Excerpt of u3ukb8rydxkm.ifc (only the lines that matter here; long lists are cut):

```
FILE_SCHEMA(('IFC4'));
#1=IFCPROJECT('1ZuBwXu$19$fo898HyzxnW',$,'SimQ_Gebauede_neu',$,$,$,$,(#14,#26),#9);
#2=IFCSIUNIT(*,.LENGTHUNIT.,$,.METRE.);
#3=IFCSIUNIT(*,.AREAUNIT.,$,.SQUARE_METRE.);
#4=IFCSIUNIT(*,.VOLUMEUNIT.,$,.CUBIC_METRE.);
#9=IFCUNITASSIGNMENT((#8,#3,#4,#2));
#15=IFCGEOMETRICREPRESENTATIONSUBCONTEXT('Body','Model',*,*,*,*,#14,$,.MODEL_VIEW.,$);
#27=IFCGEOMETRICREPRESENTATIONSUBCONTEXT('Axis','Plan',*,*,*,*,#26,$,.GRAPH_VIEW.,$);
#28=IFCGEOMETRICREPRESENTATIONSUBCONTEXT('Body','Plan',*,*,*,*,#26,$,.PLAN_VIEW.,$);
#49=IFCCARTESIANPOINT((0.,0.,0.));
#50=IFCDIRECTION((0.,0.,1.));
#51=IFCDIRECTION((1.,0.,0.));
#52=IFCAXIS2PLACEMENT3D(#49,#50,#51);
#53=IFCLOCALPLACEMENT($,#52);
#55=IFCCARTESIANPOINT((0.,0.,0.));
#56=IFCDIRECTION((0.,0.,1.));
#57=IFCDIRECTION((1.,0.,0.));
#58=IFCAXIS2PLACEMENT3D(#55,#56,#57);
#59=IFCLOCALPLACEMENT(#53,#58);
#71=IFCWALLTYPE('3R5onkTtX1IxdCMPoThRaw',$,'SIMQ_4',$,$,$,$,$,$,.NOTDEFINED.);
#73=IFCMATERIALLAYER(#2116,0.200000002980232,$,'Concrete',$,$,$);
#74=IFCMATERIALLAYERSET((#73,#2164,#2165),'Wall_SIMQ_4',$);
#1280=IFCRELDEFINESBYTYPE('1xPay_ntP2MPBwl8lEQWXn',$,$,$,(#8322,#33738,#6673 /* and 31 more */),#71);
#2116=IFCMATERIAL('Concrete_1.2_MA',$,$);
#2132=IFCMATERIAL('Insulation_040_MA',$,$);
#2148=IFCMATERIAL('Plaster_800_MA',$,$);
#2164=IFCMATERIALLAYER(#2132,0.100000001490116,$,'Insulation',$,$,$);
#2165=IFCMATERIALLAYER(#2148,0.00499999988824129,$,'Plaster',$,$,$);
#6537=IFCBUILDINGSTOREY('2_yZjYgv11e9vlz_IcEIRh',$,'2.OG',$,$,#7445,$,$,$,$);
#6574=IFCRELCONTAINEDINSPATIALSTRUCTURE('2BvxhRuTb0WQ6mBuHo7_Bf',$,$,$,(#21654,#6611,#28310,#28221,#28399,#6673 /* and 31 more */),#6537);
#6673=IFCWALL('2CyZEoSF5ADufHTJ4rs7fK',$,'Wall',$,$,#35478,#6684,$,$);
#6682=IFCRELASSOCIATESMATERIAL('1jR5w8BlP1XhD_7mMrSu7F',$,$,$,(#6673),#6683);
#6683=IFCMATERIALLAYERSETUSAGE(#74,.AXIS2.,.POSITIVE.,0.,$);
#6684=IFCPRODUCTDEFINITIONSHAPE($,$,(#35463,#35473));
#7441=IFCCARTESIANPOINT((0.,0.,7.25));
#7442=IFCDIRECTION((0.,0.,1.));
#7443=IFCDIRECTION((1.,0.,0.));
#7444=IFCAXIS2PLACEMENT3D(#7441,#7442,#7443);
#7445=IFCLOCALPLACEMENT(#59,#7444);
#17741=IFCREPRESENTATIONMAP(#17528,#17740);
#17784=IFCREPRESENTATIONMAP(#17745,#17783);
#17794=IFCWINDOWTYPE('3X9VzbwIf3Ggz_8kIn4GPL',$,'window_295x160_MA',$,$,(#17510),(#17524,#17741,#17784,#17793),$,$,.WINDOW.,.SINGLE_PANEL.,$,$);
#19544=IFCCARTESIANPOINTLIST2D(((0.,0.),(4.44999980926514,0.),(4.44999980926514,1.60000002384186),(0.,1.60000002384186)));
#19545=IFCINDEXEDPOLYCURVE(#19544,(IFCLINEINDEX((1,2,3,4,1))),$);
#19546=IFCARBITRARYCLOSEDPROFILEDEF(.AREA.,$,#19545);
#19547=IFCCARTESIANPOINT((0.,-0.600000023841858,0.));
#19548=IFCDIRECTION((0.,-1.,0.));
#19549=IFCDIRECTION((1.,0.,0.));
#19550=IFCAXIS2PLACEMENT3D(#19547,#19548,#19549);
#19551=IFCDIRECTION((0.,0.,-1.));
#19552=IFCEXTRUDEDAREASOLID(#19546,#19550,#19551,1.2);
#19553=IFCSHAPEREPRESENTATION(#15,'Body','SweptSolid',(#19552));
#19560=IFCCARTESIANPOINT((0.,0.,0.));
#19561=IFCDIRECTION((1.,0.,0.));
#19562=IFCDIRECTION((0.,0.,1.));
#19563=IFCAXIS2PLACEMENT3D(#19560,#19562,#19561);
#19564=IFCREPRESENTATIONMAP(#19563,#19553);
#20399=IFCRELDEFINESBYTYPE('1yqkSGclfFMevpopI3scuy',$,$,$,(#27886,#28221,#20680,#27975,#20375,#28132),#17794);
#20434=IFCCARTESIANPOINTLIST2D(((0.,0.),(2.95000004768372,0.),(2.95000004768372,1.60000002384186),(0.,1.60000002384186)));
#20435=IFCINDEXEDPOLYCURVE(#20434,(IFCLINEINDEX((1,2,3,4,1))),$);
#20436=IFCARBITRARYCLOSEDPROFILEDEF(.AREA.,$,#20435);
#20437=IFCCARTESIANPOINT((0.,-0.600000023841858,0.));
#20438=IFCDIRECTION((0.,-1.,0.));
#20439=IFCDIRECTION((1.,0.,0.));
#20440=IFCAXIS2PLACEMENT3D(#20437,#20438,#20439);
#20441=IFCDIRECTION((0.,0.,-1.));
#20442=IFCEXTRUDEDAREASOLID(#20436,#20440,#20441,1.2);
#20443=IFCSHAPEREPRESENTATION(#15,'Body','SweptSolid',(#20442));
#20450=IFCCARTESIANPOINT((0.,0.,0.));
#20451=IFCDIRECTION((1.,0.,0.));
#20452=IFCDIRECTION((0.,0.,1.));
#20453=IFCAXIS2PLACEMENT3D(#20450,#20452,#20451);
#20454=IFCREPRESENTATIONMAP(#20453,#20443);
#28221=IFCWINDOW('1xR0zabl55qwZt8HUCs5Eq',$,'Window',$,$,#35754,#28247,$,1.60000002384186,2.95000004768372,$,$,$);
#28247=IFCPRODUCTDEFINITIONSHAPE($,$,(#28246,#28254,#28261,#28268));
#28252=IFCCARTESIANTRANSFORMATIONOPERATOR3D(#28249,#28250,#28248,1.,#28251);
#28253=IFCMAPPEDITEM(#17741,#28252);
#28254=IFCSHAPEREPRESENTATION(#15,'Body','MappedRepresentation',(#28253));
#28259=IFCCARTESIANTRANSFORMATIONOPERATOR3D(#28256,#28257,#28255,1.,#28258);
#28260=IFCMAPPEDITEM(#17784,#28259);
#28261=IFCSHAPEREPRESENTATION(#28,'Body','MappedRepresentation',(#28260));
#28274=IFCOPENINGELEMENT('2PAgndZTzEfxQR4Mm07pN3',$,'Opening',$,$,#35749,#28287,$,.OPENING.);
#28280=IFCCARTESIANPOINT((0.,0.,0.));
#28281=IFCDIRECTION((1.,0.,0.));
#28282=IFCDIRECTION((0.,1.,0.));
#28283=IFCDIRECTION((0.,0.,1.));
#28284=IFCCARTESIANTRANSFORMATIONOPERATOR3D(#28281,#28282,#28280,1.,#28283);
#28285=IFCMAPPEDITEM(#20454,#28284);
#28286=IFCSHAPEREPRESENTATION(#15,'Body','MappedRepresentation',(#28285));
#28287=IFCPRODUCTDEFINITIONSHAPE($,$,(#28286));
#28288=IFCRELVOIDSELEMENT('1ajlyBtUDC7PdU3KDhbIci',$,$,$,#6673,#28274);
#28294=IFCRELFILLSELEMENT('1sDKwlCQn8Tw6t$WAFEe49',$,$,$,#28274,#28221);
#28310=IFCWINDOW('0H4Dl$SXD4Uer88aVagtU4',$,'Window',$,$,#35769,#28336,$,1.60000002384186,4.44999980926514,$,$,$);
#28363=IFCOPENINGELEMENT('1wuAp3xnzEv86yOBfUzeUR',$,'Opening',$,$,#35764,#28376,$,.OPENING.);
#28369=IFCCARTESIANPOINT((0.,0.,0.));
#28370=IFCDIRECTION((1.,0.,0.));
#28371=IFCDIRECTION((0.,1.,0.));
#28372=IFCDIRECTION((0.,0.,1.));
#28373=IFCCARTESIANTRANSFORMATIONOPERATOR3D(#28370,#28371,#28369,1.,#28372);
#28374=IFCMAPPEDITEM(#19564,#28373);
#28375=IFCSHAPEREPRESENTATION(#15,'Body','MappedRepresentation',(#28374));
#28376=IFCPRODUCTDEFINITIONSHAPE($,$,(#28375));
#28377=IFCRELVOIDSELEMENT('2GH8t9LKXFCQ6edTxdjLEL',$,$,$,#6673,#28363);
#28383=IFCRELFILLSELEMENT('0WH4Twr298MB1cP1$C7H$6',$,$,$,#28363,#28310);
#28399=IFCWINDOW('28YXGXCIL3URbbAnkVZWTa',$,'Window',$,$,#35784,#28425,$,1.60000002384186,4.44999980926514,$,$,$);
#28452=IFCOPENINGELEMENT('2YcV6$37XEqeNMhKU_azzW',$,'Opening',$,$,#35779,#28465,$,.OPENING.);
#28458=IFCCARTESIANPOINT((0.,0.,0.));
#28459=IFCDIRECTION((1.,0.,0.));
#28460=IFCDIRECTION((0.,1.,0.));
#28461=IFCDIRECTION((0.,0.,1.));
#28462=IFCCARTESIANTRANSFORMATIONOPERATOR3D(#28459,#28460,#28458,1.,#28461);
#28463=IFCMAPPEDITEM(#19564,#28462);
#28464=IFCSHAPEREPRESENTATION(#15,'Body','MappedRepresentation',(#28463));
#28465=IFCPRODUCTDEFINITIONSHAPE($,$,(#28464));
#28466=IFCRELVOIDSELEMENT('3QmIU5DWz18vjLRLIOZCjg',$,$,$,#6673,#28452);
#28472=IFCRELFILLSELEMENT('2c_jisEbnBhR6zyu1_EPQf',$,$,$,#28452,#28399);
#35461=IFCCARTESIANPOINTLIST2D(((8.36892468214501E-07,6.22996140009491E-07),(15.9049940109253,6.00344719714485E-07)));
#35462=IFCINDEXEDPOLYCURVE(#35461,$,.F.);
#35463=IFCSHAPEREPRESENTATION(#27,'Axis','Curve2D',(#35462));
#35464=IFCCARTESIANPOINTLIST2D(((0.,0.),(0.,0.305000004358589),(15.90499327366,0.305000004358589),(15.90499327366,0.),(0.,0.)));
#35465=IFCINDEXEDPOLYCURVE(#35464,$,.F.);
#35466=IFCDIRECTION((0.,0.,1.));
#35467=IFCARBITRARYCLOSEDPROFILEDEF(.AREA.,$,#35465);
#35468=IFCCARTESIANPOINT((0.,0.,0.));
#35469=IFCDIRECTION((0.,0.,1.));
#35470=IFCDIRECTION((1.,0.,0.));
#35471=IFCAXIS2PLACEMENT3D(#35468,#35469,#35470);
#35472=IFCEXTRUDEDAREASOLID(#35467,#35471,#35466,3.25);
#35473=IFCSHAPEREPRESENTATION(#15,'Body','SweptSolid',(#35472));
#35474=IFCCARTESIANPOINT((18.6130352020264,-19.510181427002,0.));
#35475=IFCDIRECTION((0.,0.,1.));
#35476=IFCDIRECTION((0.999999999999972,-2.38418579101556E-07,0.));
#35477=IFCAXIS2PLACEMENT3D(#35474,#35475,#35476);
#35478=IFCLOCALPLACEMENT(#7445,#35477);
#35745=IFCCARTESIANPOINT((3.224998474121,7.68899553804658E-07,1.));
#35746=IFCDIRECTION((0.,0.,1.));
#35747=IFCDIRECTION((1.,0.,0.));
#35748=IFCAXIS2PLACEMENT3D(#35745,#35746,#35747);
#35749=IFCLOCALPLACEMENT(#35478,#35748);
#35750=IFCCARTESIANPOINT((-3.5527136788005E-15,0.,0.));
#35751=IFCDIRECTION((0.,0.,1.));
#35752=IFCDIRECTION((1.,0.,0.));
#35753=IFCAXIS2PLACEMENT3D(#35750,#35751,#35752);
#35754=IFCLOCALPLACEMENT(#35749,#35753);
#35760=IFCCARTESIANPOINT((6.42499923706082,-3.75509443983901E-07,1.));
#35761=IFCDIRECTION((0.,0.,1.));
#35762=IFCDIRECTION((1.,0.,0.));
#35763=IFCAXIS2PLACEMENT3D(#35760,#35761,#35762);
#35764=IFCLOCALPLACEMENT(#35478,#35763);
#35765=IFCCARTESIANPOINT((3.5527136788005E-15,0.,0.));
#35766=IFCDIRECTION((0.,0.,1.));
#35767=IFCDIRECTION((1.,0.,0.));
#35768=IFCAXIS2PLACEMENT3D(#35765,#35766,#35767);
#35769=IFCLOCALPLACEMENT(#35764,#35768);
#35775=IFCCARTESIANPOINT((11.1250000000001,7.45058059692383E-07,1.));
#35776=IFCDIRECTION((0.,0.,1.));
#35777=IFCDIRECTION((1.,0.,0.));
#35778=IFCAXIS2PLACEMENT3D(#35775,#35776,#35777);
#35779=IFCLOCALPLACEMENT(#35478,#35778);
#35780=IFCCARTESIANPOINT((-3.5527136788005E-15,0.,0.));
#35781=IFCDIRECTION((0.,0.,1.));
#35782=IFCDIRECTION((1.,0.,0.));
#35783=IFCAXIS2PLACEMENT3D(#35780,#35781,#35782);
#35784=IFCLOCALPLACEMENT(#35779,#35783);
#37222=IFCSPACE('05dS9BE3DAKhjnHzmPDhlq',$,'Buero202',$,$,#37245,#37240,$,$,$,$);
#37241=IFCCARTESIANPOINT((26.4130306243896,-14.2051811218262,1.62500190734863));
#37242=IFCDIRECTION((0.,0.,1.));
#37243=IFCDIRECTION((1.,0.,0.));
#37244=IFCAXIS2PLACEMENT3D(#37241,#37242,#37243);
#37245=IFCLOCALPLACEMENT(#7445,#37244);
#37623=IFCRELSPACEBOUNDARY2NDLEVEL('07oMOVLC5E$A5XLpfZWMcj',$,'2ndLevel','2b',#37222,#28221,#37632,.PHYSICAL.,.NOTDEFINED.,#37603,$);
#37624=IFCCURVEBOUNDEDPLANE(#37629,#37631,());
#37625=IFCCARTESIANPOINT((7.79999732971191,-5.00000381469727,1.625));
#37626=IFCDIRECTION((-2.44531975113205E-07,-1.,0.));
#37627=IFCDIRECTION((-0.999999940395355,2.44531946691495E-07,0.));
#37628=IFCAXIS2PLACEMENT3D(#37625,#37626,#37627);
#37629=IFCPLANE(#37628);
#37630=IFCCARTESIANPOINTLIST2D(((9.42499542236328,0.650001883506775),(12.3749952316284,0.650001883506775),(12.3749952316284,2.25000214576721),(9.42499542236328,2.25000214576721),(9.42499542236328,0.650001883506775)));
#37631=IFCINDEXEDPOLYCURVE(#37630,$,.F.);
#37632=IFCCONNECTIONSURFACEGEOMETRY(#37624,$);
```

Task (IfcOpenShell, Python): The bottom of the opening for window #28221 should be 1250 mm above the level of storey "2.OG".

```python
import numpy as np
import ifcopenshell
import ifcopenshell.api.geometry
import ifcopenshell.geom
import ifcopenshell.util.element
import ifcopenshell.util.placement
import ifcopenshell.util.shape
import ifcopenshell.util.unit

model = ifcopenshell.open("u3ukb8rydxkm.ifc")
unit_scale = ifcopenshell.util.unit.calculate_unit_scale(model)

window = model.by_guid("1xR0zabl55qwZt8HUCs5Eq")
opening = window.FillsVoids[0].RelatingOpeningElement
storey = ifcopenshell.util.element.get_container(window, ifc_class="IfcBuildingStorey")
level = ifcopenshell.util.placement.get_local_placement(storey.ObjectPlacement)[2, 3]

# The opening's origin need not be at the sill, so measure its lowest point.
shape = ifcopenshell.geom.create_shape(ifcopenshell.geom.settings(), opening)
bottom = ifcopenshell.util.shape.get_shape_bottom_elevation(shape, shape.geometry) / unit_scale
dz = level + 1.25 - bottom

shift = np.array([0.0, 0.0, dz])
# The window is placed relative to its opening, so it follows when the opening moves.
matrix = ifcopenshell.util.placement.get_local_placement(opening.ObjectPlacement)
matrix[:3, 3] += shift
ifcopenshell.api.geometry.edit_object_placement(
    model, product=opening, matrix=matrix, is_si=False, should_transform_children=True
)

# Space boundary surfaces are stored in each space's coordinates; move them too.
for rel in window.ProvidesBoundaries:
    if not rel.ConnectionGeometry:
        continue
    surface = rel.ConnectionGeometry.SurfaceOnRelatingElement.BasisSurface
    space_matrix = ifcopenshell.util.placement.get_local_placement(rel.RelatingSpace.ObjectPlacement)
    point = np.array(surface.Position.Location.Coordinates) + space_matrix[:3, :3].T @ shift
    surface.Position = model.createIfcAxis2Placement3D(
        model.createIfcCartesianPoint(point.tolist()), surface.Position.Axis, surface.Position.RefDirection
    )

print(f"moved by {dz * unit_scale:+.3f} m")

model.write("u3ukb8rydxkm_v2.ifc")
```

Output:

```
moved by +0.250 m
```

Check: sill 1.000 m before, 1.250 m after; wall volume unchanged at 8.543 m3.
